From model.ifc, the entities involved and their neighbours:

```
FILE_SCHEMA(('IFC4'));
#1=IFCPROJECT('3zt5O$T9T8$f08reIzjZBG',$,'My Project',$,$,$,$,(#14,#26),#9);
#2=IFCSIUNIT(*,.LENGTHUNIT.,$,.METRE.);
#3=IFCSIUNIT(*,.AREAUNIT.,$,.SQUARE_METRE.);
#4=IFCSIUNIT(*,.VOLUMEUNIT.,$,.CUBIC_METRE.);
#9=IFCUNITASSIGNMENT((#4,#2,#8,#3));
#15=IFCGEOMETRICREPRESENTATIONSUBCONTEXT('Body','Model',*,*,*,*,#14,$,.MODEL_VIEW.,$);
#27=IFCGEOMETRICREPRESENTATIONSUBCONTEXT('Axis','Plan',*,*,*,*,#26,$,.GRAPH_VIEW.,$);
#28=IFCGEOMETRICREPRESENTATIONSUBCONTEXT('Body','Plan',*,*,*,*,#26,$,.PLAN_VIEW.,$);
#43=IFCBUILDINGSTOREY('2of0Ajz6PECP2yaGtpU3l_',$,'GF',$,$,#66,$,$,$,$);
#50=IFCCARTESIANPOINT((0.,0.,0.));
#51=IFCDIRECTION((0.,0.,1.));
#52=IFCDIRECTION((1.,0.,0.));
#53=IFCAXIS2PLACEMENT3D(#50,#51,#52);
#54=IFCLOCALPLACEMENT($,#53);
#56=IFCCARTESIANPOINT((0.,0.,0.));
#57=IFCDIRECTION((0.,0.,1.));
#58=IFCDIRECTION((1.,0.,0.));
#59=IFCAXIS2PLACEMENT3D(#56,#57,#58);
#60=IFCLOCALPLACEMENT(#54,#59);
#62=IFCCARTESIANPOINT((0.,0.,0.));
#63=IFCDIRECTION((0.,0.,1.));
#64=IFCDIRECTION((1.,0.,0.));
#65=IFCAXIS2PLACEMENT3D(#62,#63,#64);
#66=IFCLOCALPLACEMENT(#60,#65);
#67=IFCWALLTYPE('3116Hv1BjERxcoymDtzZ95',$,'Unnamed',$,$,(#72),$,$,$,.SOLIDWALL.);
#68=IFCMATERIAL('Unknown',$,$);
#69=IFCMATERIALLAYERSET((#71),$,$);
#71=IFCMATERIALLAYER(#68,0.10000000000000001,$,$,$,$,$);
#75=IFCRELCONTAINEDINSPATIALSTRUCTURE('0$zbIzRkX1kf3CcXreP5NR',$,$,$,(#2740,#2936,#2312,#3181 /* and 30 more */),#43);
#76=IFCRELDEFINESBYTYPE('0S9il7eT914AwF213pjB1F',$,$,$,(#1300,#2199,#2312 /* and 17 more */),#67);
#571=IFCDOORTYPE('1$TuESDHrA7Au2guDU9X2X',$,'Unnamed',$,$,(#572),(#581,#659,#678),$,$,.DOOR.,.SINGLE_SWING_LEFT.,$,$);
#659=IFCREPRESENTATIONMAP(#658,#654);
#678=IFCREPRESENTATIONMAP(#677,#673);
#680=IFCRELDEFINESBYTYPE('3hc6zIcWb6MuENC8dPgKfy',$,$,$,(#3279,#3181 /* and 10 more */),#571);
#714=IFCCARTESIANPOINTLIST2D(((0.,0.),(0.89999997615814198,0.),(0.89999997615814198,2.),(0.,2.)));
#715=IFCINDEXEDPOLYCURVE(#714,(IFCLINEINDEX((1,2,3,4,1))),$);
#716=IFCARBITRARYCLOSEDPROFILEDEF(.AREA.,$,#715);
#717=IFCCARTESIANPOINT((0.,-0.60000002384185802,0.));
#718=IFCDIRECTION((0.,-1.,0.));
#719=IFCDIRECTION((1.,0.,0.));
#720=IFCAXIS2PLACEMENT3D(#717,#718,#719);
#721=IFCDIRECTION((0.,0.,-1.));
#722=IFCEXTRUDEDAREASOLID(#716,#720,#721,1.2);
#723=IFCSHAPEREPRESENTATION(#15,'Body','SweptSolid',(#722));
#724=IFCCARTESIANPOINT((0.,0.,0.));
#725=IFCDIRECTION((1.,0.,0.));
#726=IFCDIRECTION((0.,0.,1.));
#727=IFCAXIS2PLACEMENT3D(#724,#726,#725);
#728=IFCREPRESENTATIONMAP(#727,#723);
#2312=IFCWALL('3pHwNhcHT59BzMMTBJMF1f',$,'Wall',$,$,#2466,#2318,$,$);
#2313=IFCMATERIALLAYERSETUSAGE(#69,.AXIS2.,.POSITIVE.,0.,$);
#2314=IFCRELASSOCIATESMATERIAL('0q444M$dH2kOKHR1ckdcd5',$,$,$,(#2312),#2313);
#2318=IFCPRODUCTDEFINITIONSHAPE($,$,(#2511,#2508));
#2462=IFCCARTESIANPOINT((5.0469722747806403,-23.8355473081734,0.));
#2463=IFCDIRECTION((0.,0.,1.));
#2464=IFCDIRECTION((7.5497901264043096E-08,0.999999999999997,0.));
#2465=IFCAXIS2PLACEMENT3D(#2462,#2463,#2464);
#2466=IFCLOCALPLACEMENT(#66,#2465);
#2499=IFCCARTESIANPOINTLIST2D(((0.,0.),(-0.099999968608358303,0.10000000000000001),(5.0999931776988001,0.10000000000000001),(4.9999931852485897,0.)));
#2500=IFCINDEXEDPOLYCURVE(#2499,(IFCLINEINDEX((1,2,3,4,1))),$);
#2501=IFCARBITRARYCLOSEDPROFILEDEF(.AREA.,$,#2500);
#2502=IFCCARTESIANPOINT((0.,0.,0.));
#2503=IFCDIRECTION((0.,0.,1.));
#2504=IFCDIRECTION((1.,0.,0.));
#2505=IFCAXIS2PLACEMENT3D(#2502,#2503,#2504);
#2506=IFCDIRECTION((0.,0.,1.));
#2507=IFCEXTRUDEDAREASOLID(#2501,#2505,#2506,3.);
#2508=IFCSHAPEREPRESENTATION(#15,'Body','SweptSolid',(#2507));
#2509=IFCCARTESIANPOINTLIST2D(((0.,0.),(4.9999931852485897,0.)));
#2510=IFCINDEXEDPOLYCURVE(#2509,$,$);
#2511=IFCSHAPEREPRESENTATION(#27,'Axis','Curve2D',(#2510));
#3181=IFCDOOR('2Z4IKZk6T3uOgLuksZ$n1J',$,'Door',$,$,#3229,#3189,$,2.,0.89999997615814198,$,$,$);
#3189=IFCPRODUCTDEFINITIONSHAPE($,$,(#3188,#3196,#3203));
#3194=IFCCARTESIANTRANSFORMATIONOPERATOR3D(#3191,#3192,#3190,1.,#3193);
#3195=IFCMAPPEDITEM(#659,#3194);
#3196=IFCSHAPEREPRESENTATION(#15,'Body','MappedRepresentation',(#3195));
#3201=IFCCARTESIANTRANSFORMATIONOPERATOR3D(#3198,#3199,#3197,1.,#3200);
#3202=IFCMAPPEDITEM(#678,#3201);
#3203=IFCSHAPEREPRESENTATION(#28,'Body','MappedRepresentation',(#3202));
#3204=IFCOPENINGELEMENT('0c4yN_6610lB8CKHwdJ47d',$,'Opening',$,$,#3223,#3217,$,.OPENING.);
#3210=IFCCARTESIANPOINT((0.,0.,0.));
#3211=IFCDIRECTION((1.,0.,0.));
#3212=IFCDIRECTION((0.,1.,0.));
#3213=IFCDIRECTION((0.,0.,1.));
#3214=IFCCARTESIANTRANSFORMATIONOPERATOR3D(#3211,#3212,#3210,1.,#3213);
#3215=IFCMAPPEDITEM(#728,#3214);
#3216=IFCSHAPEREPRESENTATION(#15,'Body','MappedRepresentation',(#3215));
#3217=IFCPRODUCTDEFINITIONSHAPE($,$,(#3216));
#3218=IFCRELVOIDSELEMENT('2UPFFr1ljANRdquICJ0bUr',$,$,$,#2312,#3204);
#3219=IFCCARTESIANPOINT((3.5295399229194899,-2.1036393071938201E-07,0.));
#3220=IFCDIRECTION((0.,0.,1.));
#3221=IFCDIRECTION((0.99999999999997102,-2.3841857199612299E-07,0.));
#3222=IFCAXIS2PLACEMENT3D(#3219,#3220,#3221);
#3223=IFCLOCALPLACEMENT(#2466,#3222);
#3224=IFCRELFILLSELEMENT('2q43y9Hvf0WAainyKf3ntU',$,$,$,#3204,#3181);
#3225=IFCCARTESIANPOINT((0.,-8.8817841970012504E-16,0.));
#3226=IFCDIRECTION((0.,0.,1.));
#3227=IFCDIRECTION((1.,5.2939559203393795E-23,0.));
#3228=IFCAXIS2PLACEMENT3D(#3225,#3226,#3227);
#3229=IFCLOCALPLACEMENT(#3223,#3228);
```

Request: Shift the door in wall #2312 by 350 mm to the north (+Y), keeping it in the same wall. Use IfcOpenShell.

```python
import ifcopenshell
import ifcopenshell.api.geometry
import ifcopenshell.util.placement
import ifcopenshell.util.unit

model = ifcopenshell.open("model.ifc")
unit_scale = ifcopenshell.util.unit.calculate_unit_scale(model)

door = model.by_guid("2Z4IKZk6T3uOgLuksZ$n1J")
opening = door.FillsVoids[0].RelatingOpeningElement
wall = opening.VoidsElements[0].RelatingBuildingElement

wall_matrix = ifcopenshell.util.placement.get_local_placement(wall.ObjectPlacement)
shift = wall_matrix[:3, 0] * 0.35 / unit_scale
before = ifcopenshell.util.placement.get_local_placement(door.ObjectPlacement)[:3, 3].copy()

# The door is placed relative to its opening, so it follows when the opening moves.
matrix = ifcopenshell.util.placement.get_local_placement(opening.ObjectPlacement)
matrix[:3, 3] += shift
ifcopenshell.api.geometry.edit_object_placement(
    model, product=opening, matrix=matrix, is_si=False, should_transform_children=True
)

after = ifcopenshell.util.placement.get_local_placement(door.ObjectPlacement)[:3, 3]
print("door moved by", (after - before).round(3) + 0.0)

model.write("model_v2.ifc")
```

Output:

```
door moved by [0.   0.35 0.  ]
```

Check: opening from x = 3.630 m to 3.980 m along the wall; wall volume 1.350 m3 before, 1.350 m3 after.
